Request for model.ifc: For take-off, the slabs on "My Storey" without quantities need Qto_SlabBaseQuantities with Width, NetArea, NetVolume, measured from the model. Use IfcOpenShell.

First a look at what the model holds.

```python
import ifcopenshell
import ifcopenshell.util.element
import ifcopenshell.util.unit

model = ifcopenshell.open("model.ifc")
print(model.schema)
for unit_type in ("LENGTHUNIT", "AREAUNIT", "VOLUMEUNIT"):
    print(unit_type, ifcopenshell.util.unit.calculate_unit_scale(model, unit_type))
storey = next(s for s in model.by_type("IfcBuildingStorey") if s.Name == "My Storey")
slabs = [e for e in ifcopenshell.util.element.get_decomposition(storey) if e.is_a("IfcSlab")]
for e in sorted(slabs, key=lambda e: e.id()):
    print(e.id(), e.is_a(), e.Name, list(ifcopenshell.util.element.get_psets(e, qtos_only=True)), sep=" | ")
```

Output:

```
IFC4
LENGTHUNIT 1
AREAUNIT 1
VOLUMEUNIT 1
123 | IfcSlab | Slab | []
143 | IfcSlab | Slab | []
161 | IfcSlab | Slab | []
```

```python
import ifcopenshell
import ifcopenshell.api.pset
import ifcopenshell.geom
import ifcopenshell.util.element
import ifcopenshell.util.shape
import ifcopenshell.util.unit

model = ifcopenshell.open("model.ifc")
unit_scale = ifcopenshell.util.unit.calculate_unit_scale(model)
area_scale = ifcopenshell.util.unit.calculate_unit_scale(model, "AREAUNIT")
volume_scale = ifcopenshell.util.unit.calculate_unit_scale(model, "VOLUMEUNIT")
settings = ifcopenshell.geom.settings()

storey = next(s for s in model.by_type("IfcBuildingStorey") if s.Name == "My Storey")
slabs = [e for e in ifcopenshell.util.element.get_decomposition(storey) if e.is_a("IfcSlab")]

for e in sorted(slabs, key=lambda e: e.id()):
    if ifcopenshell.util.element.get_psets(e, qtos_only=True, should_inherit=False):
        continue
    # Geometry comes back in metres, in the element's own axes.
    shape = ifcopenshell.geom.create_shape(settings, e)
    values = {
        "Width": ifcopenshell.util.shape.get_z(shape.geometry) / unit_scale,
        "NetArea": ifcopenshell.util.shape.get_footprint_area(shape.geometry) / area_scale,
        "NetVolume": ifcopenshell.util.shape.get_volume(shape.geometry) / volume_scale,
    }
    qto = ifcopenshell.api.pset.add_qto(model, product=e, name="Qto_SlabBaseQuantities")
    ifcopenshell.api.pset.edit_qto(model, qto=qto, properties=values)
    print(e.id(), {k: round(v, 3) for k, v in values.items()})

model.write("model_edited.ifc")
```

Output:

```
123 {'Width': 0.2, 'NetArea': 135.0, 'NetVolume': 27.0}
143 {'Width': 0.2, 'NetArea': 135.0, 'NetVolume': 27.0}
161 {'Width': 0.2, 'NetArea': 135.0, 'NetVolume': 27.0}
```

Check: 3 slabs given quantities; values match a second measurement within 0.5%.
